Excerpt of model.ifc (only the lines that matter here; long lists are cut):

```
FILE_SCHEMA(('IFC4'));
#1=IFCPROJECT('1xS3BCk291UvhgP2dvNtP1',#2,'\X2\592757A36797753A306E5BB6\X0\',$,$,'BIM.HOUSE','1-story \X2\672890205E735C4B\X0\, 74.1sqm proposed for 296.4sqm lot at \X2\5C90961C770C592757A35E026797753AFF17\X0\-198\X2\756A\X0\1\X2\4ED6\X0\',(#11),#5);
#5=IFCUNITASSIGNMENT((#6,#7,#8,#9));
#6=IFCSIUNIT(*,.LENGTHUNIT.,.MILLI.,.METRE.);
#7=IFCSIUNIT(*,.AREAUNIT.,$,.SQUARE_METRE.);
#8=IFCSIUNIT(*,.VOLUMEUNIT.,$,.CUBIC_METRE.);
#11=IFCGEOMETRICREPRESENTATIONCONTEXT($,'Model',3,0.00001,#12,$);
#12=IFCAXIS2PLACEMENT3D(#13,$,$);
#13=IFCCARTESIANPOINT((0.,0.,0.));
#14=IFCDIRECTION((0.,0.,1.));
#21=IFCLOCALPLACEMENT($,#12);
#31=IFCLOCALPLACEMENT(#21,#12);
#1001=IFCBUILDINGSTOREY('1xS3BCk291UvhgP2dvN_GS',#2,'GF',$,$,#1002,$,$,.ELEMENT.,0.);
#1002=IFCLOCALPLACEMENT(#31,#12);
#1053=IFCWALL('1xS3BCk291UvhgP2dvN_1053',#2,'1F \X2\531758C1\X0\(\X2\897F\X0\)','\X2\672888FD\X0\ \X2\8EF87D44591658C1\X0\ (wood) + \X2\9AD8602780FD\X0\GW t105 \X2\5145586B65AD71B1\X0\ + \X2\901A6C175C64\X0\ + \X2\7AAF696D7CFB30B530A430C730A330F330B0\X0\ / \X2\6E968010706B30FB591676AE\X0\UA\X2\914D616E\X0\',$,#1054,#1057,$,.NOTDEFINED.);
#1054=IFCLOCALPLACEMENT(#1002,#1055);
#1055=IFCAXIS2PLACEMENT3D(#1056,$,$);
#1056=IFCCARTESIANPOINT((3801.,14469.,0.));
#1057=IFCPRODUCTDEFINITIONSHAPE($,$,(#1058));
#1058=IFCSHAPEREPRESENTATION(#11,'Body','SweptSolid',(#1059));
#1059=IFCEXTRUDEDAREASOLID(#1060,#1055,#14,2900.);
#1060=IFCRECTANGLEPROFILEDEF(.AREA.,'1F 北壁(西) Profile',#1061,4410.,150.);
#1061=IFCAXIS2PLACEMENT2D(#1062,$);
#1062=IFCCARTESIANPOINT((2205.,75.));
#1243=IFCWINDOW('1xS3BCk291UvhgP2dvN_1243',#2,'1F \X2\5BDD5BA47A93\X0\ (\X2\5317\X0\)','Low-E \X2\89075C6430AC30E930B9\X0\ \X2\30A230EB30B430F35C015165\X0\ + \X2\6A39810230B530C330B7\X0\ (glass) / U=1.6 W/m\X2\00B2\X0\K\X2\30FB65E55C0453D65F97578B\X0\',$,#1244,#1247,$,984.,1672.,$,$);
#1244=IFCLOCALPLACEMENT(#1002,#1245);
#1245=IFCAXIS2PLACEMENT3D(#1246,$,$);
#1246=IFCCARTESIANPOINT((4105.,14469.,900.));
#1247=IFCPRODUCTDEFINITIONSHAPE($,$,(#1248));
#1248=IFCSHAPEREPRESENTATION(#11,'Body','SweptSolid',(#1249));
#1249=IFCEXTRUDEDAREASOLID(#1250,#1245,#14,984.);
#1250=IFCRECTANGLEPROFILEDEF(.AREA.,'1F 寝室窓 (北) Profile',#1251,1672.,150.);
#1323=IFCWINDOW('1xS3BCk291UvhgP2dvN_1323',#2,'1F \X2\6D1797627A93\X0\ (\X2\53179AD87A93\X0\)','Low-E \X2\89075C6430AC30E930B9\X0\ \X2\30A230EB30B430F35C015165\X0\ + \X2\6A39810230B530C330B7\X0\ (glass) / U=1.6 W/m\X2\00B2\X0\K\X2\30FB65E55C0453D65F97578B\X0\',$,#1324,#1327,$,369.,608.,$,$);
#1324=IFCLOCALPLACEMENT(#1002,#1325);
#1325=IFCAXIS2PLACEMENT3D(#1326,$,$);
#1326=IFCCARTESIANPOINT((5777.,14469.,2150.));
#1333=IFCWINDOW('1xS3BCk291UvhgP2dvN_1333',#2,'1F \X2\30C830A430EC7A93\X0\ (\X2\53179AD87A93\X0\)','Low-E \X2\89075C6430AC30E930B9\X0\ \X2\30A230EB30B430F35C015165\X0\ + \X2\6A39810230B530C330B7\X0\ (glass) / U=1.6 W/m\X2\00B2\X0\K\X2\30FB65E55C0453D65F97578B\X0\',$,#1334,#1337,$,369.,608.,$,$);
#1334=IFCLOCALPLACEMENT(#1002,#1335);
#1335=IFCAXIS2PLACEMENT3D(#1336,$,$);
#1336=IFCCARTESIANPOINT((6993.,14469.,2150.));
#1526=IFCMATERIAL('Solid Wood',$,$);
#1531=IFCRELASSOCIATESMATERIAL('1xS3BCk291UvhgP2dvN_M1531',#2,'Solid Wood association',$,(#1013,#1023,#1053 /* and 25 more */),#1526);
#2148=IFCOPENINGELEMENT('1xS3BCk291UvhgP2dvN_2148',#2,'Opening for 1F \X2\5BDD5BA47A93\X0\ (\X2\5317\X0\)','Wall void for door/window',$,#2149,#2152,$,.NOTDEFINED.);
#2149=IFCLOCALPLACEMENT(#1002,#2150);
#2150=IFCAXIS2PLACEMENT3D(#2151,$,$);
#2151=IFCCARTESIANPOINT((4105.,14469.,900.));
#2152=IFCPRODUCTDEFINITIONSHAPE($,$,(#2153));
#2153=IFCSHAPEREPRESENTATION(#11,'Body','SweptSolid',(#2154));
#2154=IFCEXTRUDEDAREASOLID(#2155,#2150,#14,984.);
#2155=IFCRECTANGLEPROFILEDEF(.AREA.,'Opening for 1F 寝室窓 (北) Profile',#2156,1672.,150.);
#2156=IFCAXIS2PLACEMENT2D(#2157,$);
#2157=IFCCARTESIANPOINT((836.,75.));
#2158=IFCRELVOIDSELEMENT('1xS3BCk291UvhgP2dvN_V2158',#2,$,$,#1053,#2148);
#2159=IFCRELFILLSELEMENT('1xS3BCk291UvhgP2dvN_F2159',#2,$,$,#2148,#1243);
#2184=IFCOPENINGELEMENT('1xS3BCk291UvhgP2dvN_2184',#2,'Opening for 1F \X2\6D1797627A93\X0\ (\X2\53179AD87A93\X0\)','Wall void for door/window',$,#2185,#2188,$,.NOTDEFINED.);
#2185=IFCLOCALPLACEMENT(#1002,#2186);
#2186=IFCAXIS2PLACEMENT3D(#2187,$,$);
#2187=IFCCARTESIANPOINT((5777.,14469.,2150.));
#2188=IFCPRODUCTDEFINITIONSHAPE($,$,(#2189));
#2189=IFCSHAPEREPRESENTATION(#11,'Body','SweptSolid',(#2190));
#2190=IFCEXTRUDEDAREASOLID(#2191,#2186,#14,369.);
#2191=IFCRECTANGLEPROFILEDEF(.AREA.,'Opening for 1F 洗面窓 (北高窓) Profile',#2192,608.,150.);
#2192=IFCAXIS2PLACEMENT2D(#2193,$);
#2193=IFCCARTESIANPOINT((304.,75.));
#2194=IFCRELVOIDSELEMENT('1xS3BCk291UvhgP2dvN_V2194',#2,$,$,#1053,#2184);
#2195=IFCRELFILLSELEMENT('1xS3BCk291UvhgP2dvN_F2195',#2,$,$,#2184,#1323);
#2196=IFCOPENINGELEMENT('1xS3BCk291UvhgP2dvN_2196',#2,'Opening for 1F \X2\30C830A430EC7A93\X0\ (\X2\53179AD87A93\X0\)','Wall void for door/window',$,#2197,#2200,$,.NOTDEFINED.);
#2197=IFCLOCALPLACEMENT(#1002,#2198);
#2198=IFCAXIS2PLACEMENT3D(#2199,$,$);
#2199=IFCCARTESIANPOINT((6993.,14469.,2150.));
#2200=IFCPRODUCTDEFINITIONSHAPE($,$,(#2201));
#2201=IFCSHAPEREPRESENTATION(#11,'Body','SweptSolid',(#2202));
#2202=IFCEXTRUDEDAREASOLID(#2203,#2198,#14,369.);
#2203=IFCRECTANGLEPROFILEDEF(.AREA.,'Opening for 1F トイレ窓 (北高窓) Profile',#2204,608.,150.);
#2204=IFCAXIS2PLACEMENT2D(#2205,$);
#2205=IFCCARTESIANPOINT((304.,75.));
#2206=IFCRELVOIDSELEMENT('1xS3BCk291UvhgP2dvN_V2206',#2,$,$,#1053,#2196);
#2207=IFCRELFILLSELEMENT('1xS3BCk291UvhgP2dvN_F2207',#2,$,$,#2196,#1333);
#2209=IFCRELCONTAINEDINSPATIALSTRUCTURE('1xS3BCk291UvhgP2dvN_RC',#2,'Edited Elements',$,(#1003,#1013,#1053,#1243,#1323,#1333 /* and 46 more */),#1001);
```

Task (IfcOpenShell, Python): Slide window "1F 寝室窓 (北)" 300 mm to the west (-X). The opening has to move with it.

```python
import ifcopenshell
import ifcopenshell.api.geometry
import ifcopenshell.util.placement
import ifcopenshell.util.unit

model = ifcopenshell.open("model.ifc")
unit_scale = ifcopenshell.util.unit.calculate_unit_scale(model)

window = model.by_guid("1xS3BCk291UvhgP2dvN_1243")
opening = window.FillsVoids[0].RelatingOpeningElement
wall = opening.VoidsElements[0].RelatingBuildingElement

wall_matrix = ifcopenshell.util.placement.get_local_placement(wall.ObjectPlacement)
shift = wall_matrix[:3, 0] * -0.3 / unit_scale
before = ifcopenshell.util.placement.get_local_placement(window.ObjectPlacement)[:3, 3].copy()

# The window is not placed relative to its opening, so move both.
for product in (opening, window):
    matrix = ifcopenshell.util.placement.get_local_placement(product.ObjectPlacement)
    matrix[:3, 3] += shift
    ifcopenshell.api.geometry.edit_object_placement(model, product=product, matrix=matrix, is_si=False)

after = ifcopenshell.util.placement.get_local_placement(window.ObjectPlacement)[:3, 3]
print("window moved by", (after - before).round(3) + 0.0)

model.write("model-out.ifc")
```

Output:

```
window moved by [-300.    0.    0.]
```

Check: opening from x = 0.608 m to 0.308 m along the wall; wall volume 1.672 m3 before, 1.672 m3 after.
